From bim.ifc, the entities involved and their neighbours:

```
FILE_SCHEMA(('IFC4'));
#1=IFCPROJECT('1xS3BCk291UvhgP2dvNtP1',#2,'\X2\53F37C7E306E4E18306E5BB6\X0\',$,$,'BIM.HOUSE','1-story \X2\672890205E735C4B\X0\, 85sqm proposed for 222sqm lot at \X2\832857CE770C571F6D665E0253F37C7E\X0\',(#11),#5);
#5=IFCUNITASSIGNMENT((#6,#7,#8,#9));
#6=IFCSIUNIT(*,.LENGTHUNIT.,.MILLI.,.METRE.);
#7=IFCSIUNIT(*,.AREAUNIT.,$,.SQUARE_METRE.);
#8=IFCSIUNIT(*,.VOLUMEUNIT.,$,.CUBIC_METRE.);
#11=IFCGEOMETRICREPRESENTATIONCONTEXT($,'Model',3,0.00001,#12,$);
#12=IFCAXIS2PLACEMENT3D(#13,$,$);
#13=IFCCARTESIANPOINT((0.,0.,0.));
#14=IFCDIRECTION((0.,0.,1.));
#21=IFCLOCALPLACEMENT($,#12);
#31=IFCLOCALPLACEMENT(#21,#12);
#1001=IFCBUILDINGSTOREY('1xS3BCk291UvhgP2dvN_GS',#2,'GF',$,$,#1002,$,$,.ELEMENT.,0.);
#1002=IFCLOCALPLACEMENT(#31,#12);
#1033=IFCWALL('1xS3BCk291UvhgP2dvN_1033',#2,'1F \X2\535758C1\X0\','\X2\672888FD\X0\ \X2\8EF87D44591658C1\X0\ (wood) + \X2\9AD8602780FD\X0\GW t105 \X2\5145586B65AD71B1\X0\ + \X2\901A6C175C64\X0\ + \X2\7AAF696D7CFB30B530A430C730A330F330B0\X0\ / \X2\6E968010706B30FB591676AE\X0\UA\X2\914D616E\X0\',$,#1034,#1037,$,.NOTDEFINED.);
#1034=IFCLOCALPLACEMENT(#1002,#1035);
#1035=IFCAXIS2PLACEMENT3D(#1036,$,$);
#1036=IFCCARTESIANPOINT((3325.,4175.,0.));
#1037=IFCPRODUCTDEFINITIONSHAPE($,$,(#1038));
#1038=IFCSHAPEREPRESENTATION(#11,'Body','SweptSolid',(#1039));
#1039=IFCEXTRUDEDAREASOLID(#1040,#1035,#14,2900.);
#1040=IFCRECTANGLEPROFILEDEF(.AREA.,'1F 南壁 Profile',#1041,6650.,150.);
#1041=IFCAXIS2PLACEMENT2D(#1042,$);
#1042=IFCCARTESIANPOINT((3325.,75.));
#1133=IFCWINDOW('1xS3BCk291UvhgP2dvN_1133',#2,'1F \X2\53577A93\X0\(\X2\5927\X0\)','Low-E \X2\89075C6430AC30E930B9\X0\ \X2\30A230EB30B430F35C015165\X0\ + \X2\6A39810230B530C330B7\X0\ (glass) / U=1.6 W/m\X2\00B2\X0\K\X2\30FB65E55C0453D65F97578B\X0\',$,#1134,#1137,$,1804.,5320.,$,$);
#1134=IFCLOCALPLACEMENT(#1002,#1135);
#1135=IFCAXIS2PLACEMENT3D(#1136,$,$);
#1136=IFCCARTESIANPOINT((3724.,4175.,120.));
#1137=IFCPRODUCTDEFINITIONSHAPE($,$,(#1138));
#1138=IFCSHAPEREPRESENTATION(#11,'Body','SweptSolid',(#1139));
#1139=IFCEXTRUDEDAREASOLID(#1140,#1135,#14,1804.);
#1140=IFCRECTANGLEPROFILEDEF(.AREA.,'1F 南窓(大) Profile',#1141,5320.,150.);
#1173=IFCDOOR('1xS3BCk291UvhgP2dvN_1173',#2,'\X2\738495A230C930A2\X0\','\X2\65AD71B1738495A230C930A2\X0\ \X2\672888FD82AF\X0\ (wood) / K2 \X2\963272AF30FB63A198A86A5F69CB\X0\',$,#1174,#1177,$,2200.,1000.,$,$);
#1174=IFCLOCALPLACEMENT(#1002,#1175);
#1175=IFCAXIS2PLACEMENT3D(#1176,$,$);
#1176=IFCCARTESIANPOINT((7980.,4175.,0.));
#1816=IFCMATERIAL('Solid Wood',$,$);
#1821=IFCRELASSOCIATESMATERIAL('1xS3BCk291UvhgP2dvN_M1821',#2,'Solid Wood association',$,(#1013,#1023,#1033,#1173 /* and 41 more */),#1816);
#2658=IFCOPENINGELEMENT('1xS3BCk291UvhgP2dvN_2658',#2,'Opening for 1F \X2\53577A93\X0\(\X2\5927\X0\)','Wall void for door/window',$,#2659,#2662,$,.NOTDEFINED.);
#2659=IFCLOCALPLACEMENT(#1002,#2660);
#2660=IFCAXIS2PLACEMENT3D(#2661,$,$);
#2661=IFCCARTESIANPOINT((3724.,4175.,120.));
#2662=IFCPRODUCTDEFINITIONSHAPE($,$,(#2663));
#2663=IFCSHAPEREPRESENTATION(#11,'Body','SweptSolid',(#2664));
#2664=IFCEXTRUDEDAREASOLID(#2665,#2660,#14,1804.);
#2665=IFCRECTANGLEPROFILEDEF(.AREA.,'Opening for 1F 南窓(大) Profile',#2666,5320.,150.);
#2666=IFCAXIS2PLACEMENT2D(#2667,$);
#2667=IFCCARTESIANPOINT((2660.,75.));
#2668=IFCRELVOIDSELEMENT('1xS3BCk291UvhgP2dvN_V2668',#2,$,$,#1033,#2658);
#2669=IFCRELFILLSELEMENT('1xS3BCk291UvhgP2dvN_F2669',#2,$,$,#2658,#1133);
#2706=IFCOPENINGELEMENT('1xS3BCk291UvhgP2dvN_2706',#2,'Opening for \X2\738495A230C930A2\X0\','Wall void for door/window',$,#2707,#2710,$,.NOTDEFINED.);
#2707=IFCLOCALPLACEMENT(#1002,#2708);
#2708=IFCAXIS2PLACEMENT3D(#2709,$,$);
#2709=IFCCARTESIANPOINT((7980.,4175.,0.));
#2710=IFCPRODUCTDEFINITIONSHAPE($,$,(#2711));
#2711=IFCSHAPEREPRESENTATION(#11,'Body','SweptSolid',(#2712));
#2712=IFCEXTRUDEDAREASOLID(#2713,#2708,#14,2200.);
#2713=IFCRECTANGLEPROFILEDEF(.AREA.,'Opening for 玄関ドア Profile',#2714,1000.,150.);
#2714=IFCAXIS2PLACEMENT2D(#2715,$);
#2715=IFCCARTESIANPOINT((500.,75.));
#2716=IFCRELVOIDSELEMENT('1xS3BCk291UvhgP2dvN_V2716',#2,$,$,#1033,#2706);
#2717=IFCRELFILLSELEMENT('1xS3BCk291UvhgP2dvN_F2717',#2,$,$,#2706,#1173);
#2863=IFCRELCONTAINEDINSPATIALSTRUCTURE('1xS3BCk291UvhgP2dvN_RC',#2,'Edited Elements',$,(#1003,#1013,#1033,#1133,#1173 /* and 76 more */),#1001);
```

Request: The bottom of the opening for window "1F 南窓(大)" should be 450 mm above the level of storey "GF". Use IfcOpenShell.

```python
import numpy as np
import ifcopenshell
import ifcopenshell.api.geometry
import ifcopenshell.geom
import ifcopenshell.util.element
import ifcopenshell.util.placement
import ifcopenshell.util.shape
import ifcopenshell.util.unit

model = ifcopenshell.open("bim.ifc")
unit_scale = ifcopenshell.util.unit.calculate_unit_scale(model)

window = model.by_id(1133)
opening = window.FillsVoids[0].RelatingOpeningElement
storey = ifcopenshell.util.element.get_container(window, ifc_class="IfcBuildingStorey")
level = ifcopenshell.util.placement.get_local_placement(storey.ObjectPlacement)[2, 3]

# The opening's origin need not be at the sill, so measure its lowest point.
shape = ifcopenshell.geom.create_shape(ifcopenshell.geom.settings(), opening)
bottom = ifcopenshell.util.shape.get_shape_bottom_elevation(shape, shape.geometry) / unit_scale
dz = level + 0.45 / unit_scale - bottom

shift = np.array([0.0, 0.0, dz])
# The window is not placed relative to its opening, so move both.
for product in (opening, window):
    matrix = ifcopenshell.util.placement.get_local_placement(product.ObjectPlacement)
    matrix[:3, 3] += shift
    ifcopenshell.api.geometry.edit_object_placement(model, product=product, matrix=matrix, is_si=False)

print(f"moved by {dz * unit_scale:+.3f} m")

model.write("bim_edited.ifc")
```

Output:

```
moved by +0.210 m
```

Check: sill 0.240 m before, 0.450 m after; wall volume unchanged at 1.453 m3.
